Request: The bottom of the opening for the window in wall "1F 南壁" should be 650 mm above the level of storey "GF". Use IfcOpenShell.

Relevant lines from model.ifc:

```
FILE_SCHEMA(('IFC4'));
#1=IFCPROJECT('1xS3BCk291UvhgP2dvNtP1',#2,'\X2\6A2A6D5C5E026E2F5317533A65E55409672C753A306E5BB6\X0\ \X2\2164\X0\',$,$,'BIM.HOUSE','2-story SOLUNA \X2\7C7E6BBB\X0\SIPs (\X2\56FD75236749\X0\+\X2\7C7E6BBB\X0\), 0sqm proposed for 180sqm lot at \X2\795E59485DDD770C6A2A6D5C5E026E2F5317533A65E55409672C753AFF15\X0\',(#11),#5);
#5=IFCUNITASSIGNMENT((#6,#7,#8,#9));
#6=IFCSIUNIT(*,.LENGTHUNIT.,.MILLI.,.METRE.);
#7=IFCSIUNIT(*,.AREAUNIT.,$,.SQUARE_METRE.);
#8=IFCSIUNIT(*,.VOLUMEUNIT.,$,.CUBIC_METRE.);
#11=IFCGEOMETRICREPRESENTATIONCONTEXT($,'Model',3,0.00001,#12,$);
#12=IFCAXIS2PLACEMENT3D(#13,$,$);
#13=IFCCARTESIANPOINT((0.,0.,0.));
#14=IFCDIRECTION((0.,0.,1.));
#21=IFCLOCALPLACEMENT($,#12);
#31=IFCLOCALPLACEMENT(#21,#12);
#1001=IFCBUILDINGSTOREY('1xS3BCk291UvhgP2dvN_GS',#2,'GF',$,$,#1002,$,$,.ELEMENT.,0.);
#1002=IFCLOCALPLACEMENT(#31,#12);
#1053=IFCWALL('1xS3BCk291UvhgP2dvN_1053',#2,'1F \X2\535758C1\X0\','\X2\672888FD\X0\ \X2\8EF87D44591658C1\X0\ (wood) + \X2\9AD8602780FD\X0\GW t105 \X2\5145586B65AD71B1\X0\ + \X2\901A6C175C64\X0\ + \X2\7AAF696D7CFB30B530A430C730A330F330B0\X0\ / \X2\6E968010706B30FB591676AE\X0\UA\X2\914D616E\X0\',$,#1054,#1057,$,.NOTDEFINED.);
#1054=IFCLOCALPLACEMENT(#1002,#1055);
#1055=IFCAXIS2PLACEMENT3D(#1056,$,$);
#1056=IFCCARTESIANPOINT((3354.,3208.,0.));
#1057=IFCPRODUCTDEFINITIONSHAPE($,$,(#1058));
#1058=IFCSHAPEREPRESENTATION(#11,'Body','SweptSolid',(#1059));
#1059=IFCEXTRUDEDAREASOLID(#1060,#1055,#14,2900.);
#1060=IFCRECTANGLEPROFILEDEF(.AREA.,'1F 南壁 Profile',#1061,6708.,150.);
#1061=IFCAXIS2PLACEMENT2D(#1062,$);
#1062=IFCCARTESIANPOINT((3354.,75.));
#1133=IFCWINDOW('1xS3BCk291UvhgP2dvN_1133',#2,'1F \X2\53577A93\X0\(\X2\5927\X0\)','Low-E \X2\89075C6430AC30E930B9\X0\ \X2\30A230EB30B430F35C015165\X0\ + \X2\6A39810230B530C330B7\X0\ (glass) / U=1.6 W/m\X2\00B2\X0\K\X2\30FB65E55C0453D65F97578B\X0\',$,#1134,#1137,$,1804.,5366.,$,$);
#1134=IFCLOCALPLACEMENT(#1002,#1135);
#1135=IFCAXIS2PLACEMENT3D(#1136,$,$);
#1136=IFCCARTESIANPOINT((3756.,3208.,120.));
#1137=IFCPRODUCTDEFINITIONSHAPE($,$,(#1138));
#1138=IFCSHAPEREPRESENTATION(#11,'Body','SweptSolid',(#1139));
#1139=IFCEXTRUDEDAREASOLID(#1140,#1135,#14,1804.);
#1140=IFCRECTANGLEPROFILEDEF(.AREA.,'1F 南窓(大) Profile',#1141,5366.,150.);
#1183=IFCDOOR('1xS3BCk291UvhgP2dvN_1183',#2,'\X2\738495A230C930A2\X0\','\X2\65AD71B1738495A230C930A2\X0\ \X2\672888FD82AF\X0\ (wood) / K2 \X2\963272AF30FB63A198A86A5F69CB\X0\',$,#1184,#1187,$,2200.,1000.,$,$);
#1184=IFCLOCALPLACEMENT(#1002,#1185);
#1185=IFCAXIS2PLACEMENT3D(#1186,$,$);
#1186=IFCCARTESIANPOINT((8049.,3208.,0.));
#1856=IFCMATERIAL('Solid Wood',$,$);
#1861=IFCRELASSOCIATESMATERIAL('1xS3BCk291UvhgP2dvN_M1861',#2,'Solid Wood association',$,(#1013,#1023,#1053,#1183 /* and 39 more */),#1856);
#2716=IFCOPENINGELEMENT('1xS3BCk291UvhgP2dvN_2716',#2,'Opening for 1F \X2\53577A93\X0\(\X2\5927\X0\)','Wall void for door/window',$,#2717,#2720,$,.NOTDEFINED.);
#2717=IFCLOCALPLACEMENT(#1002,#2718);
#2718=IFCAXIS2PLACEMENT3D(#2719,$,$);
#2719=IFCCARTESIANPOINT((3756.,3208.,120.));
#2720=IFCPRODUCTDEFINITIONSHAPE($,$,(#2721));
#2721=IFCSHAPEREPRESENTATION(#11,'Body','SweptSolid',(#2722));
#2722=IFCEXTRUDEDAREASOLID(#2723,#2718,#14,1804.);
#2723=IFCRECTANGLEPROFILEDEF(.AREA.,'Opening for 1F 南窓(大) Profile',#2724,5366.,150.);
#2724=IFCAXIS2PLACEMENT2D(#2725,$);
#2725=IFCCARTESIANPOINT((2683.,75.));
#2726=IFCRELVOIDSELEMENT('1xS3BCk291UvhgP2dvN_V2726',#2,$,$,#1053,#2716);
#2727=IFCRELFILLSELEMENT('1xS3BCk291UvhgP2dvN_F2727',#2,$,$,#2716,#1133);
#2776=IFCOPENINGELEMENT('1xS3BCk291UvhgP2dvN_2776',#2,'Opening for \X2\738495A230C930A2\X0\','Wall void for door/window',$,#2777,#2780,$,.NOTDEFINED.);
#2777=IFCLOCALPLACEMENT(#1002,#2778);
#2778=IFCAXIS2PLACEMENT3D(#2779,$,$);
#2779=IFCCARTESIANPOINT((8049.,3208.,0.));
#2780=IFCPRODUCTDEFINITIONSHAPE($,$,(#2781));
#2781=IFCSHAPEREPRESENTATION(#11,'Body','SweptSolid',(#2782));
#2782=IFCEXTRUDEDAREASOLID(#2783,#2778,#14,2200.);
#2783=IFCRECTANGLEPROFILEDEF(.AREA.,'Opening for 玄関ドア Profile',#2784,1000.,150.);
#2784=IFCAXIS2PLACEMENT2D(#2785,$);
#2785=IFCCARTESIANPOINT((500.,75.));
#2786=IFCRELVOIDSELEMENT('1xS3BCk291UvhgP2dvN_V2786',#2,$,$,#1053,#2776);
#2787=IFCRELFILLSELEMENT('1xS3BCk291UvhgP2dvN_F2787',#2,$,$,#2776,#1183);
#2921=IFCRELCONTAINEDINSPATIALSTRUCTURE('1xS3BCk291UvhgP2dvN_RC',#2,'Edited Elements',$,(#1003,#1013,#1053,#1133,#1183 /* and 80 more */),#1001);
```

```python
import numpy as np
import ifcopenshell
import ifcopenshell.api.geometry
import ifcopenshell.geom
import ifcopenshell.util.element
import ifcopenshell.util.placement
import ifcopenshell.util.shape
import ifcopenshell.util.unit

model = ifcopenshell.open("model.ifc")
unit_scale = ifcopenshell.util.unit.calculate_unit_scale(model)

window = model.by_guid("1xS3BCk291UvhgP2dvN_1133")
opening = window.FillsVoids[0].RelatingOpeningElement
storey = ifcopenshell.util.element.get_container(window, ifc_class="IfcBuildingStorey")
level = ifcopenshell.util.placement.get_local_placement(storey.ObjectPlacement)[2, 3]

# The opening's origin need not be at the sill, so measure its lowest point.
shape = ifcopenshell.geom.create_shape(ifcopenshell.geom.settings(), opening)
bottom = ifcopenshell.util.shape.get_shape_bottom_elevation(shape, shape.geometry) / unit_scale
dz = level + 650.0 - bottom

shift = np.array([0.0, 0.0, dz])
# The window is not placed relative to its opening, so move both.
for product in (opening, window):
    matrix = ifcopenshell.util.placement.get_local_placement(product.ObjectPlacement)
    matrix[:3, 3] += shift
    ifcopenshell.api.geometry.edit_object_placement(model, product=product, matrix=matrix, is_si=False)

print(f"moved by {dz * unit_scale:+.3f} m")

model.write("model-out.ifc")
```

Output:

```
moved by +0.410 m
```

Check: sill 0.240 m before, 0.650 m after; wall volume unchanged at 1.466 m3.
